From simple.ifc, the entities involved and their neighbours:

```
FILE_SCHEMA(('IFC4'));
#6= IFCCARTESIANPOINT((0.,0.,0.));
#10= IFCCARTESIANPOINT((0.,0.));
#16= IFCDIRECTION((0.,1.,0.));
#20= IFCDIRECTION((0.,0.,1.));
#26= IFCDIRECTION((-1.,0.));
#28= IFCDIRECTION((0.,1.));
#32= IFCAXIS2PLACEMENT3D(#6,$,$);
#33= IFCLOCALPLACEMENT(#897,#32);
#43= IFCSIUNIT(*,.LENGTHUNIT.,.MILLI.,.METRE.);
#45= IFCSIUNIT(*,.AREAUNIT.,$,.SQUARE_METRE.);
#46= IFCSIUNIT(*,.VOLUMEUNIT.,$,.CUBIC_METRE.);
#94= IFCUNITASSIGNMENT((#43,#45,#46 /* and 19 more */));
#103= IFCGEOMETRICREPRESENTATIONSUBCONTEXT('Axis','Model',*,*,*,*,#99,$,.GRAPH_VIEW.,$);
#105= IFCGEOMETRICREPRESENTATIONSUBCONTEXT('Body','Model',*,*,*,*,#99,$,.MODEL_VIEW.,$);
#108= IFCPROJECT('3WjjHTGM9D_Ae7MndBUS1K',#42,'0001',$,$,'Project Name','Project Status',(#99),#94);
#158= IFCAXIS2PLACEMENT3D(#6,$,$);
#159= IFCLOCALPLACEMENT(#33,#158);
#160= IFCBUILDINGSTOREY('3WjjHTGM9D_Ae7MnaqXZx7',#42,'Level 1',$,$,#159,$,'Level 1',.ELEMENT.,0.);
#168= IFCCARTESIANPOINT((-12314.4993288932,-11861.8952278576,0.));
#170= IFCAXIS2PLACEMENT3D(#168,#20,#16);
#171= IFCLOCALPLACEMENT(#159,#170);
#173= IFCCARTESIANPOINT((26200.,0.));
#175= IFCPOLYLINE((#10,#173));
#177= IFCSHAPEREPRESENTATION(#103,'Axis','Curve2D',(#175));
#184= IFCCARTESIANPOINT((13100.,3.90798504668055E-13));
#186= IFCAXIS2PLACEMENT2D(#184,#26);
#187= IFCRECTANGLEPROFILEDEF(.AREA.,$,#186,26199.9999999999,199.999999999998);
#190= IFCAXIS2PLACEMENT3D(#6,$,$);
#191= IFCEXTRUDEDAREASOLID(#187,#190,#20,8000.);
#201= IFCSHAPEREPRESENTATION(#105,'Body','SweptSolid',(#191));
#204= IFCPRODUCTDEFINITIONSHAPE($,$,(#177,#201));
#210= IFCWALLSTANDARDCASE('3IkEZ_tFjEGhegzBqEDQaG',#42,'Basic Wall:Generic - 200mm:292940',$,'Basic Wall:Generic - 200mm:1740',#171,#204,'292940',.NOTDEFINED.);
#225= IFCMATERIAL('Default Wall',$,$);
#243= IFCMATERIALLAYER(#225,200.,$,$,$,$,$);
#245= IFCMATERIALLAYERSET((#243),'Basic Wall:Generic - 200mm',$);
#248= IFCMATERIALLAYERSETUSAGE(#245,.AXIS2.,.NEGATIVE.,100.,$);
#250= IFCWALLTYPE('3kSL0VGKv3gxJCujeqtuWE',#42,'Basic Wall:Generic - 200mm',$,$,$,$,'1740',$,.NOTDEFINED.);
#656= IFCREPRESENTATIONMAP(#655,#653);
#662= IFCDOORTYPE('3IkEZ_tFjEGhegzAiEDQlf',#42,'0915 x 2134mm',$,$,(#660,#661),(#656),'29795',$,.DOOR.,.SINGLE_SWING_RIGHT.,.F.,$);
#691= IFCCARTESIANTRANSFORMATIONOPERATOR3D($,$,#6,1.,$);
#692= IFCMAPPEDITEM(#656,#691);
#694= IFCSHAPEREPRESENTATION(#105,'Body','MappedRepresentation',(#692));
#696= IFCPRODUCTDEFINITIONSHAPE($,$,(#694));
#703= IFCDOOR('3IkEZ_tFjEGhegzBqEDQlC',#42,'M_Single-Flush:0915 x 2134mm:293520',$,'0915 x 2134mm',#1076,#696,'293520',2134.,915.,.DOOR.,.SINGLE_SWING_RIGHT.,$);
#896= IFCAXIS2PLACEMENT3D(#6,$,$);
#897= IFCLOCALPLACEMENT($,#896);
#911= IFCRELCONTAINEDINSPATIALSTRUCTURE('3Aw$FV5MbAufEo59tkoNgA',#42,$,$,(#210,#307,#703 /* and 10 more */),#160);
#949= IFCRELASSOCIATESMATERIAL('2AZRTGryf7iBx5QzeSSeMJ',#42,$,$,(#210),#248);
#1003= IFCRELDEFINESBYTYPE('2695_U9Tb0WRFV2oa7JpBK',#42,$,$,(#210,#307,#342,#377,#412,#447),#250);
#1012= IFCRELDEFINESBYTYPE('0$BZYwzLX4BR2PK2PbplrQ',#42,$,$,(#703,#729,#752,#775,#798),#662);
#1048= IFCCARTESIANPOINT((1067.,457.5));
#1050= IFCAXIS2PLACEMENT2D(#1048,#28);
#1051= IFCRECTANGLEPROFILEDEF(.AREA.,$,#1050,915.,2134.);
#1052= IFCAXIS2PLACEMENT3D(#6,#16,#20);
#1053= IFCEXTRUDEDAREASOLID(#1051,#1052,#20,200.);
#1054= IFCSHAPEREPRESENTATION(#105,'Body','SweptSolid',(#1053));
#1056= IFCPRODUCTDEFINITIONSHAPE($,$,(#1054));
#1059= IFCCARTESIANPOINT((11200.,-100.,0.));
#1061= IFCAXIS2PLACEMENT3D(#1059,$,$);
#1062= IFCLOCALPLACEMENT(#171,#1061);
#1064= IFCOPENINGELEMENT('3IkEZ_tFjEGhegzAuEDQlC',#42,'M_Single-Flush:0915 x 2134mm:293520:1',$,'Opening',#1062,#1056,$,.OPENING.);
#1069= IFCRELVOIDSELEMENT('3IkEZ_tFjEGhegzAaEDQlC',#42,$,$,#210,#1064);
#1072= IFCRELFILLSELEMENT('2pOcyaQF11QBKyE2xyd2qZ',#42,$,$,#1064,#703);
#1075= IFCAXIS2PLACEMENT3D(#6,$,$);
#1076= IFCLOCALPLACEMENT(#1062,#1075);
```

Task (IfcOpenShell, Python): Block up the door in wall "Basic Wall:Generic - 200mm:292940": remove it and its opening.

```python
import ifcopenshell
import ifcopenshell.api.feature
import ifcopenshell.api.root
import ifcopenshell.geom
import ifcopenshell.util.shape

model = ifcopenshell.open("simple.ifc")
settings = ifcopenshell.geom.settings()


def volume(element):
    """Net volume in cubic metres, openings subtracted."""
    shape = ifcopenshell.geom.create_shape(settings, element)
    return ifcopenshell.util.shape.get_volume(shape.geometry)


door = model.by_id(703)
opening = door.FillsVoids[0].RelatingOpeningElement
wall = opening.VoidsElements[0].RelatingBuildingElement
before = volume(wall)

ifcopenshell.api.root.remove_product(model, product=door)
ifcopenshell.api.feature.remove_feature(model, feature=opening)

after = volume(wall)

print(f"wall volume {before:.3f} -> {after:.3f} m3")

model.write("simple_rev.ifc")
```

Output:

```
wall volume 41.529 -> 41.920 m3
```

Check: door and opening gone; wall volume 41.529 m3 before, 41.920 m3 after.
